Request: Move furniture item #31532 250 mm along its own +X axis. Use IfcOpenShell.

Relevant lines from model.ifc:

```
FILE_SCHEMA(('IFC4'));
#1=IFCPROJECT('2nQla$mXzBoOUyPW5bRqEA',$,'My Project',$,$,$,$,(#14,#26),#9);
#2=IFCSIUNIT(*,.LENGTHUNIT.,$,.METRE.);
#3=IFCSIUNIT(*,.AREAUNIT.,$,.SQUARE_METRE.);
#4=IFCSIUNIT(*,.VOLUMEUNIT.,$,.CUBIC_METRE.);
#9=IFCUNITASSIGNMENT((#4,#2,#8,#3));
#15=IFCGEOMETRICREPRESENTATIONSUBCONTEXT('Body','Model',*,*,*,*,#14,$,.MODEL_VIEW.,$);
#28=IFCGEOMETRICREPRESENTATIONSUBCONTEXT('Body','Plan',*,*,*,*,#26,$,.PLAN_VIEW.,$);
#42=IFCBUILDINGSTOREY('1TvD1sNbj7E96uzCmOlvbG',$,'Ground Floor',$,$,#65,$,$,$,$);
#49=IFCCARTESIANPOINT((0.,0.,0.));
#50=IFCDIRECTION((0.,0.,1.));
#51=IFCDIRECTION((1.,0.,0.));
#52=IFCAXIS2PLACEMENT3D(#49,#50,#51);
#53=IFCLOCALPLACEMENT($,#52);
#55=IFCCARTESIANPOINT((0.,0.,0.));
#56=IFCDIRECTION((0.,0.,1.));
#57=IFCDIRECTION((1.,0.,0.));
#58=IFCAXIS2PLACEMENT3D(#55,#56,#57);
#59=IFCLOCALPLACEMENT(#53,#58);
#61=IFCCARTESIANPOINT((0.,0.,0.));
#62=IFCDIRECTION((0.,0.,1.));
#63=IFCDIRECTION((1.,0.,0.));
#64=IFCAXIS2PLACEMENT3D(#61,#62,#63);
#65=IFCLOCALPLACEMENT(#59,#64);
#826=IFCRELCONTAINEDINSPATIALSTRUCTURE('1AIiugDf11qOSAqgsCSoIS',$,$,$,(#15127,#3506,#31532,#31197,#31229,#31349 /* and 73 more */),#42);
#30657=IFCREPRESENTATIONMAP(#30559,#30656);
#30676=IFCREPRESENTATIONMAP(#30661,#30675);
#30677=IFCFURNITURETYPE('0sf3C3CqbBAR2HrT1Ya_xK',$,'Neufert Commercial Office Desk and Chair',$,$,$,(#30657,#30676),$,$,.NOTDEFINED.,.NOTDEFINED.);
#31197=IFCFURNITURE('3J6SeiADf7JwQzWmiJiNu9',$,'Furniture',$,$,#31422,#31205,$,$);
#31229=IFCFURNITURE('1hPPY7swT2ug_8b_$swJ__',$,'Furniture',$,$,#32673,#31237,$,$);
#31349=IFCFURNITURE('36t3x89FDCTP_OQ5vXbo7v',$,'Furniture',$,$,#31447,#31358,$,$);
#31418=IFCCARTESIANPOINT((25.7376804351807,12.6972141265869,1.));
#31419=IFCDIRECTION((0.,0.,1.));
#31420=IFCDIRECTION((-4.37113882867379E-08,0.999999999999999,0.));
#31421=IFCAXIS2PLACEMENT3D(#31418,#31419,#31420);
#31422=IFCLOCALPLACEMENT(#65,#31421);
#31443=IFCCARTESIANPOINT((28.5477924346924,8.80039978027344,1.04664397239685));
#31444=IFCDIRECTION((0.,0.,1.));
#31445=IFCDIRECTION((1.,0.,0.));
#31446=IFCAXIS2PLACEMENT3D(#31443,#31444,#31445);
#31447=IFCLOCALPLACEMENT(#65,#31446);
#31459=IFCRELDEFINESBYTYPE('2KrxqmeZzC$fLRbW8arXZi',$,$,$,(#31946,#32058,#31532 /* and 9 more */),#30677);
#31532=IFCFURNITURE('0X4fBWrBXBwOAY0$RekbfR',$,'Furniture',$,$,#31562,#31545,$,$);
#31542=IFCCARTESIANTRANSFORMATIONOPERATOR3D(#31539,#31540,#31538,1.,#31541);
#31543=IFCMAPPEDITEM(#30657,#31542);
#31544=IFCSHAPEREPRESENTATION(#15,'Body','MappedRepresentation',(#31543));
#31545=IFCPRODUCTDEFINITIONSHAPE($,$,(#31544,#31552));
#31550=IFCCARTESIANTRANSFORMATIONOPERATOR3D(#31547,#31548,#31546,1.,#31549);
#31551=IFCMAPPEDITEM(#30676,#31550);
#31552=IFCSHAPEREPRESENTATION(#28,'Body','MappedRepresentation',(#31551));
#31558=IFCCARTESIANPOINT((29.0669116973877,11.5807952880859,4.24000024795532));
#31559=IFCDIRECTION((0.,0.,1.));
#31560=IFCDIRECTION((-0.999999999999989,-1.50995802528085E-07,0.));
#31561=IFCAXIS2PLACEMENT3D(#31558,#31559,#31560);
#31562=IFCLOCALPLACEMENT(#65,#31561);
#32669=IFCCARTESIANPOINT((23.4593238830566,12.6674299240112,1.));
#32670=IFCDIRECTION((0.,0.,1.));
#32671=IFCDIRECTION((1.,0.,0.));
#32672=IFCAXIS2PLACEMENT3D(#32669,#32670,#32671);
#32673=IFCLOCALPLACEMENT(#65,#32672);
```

```python
import ifcopenshell
import ifcopenshell.api.geometry
import ifcopenshell.util.placement
import ifcopenshell.util.unit

model = ifcopenshell.open("model.ifc")
unit_scale = ifcopenshell.util.unit.calculate_unit_scale(model)

item = model.by_guid("0X4fBWrBXBwOAY0$RekbfR")
matrix = ifcopenshell.util.placement.get_local_placement(item.ObjectPlacement)
matrix[:3, 3] += matrix[:3, 0] * 0.25 / unit_scale
ifcopenshell.api.geometry.edit_object_placement(model, product=item, matrix=matrix, is_si=False)

print(ifcopenshell.util.placement.get_local_placement(item.ObjectPlacement).round(3) + 0.0)

model.write("model_updated.ifc")
```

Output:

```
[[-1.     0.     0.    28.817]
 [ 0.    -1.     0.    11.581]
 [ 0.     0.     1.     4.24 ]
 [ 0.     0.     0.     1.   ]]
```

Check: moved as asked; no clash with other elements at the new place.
